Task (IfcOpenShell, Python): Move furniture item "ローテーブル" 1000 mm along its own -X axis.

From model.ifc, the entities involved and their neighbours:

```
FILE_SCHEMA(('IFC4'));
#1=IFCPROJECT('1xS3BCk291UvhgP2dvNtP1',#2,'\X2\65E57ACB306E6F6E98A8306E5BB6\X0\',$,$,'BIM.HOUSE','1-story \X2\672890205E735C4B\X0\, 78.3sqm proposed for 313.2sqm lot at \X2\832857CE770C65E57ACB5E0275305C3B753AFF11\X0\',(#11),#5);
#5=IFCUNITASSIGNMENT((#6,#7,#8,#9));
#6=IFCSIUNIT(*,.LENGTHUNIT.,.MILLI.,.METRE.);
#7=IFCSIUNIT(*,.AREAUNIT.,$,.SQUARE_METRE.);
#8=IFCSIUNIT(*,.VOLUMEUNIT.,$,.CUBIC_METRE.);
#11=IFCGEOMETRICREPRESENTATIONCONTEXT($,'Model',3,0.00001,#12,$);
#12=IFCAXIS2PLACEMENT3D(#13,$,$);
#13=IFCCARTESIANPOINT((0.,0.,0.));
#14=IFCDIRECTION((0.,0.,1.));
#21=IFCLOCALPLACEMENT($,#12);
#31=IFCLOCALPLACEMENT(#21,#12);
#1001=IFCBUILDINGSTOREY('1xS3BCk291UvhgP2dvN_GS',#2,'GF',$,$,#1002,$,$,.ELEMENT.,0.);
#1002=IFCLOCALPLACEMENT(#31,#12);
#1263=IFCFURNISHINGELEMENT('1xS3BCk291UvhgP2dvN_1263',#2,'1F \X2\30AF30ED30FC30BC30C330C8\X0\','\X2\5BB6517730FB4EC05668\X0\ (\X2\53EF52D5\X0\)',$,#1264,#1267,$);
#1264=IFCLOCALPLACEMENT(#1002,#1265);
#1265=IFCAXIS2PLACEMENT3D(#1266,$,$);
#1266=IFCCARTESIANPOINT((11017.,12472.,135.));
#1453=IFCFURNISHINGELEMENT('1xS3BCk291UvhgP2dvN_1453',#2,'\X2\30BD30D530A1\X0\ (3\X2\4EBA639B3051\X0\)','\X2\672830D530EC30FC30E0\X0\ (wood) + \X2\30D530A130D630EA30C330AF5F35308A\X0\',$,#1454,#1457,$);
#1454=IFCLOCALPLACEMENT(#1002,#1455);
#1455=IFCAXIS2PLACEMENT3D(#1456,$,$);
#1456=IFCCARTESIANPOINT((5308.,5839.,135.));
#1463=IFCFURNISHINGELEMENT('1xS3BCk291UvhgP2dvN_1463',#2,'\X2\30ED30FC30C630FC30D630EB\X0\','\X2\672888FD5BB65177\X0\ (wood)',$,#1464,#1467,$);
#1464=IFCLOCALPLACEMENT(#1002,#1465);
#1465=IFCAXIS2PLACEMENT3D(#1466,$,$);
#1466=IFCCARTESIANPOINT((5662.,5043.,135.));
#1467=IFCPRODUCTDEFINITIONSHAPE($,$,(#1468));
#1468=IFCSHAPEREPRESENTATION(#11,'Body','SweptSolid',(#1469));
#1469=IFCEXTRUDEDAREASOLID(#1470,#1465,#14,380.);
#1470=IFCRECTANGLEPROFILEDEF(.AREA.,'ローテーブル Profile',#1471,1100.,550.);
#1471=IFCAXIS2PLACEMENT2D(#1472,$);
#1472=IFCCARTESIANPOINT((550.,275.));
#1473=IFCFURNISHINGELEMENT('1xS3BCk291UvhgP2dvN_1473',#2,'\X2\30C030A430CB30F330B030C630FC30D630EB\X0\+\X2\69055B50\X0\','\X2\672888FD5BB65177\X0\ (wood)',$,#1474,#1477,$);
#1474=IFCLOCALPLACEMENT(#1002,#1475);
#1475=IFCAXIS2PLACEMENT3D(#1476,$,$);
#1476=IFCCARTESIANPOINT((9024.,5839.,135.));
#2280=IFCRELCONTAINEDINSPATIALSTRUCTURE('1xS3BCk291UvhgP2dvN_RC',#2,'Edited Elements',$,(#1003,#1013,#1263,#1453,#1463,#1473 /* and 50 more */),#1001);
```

```python
import ifcopenshell
import ifcopenshell.api.geometry
import ifcopenshell.util.placement

model = ifcopenshell.open("model.ifc")

item = model.by_guid("1xS3BCk291UvhgP2dvN_1463")
matrix = ifcopenshell.util.placement.get_local_placement(item.ObjectPlacement)
matrix[:3, 3] -= matrix[:3, 0] * 1000.0
ifcopenshell.api.geometry.edit_object_placement(model, product=item, matrix=matrix, is_si=False)

print(ifcopenshell.util.placement.get_local_placement(item.ObjectPlacement).round(3) + 0.0)

model.write("model_rev.ifc")
```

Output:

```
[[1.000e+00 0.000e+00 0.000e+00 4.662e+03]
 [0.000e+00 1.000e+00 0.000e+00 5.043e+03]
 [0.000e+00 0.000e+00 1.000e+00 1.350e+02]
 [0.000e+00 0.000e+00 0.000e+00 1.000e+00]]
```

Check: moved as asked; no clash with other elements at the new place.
